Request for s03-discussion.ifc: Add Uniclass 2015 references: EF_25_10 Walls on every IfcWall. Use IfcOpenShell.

First a look at what the model holds.

```python
import ifcopenshell

model = ifcopenshell.open("s03-discussion.ifc")
print(model.schema)
print("classifications:", [c.Name for c in model.by_type("IfcClassification")])
for ifc_class in ("IfcDoor", "IfcRoof", "IfcStair", "IfcWall", "IfcWindow"):
    print(ifc_class, len(model.by_type(ifc_class)))
```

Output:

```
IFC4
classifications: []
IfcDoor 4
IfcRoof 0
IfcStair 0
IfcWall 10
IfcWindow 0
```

```python
import ifcopenshell
import ifcopenshell.api.classification

model = ifcopenshell.open("s03-discussion.ifc")

system = ifcopenshell.api.classification.add_classification(model, classification="Uniclass 2015")

codes = {
    "IfcWall": ("EF_25_10", "Walls"),
}
for ifc_class, (code, name) in codes.items():
    products = model.by_type(ifc_class)
    ifcopenshell.api.classification.add_reference(
        model, products=products, classification=system, identification=code, name=name
    )
    print(code, len(products))

model.write("s03-discussion_edited.ifc")
```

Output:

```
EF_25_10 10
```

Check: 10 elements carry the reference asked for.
